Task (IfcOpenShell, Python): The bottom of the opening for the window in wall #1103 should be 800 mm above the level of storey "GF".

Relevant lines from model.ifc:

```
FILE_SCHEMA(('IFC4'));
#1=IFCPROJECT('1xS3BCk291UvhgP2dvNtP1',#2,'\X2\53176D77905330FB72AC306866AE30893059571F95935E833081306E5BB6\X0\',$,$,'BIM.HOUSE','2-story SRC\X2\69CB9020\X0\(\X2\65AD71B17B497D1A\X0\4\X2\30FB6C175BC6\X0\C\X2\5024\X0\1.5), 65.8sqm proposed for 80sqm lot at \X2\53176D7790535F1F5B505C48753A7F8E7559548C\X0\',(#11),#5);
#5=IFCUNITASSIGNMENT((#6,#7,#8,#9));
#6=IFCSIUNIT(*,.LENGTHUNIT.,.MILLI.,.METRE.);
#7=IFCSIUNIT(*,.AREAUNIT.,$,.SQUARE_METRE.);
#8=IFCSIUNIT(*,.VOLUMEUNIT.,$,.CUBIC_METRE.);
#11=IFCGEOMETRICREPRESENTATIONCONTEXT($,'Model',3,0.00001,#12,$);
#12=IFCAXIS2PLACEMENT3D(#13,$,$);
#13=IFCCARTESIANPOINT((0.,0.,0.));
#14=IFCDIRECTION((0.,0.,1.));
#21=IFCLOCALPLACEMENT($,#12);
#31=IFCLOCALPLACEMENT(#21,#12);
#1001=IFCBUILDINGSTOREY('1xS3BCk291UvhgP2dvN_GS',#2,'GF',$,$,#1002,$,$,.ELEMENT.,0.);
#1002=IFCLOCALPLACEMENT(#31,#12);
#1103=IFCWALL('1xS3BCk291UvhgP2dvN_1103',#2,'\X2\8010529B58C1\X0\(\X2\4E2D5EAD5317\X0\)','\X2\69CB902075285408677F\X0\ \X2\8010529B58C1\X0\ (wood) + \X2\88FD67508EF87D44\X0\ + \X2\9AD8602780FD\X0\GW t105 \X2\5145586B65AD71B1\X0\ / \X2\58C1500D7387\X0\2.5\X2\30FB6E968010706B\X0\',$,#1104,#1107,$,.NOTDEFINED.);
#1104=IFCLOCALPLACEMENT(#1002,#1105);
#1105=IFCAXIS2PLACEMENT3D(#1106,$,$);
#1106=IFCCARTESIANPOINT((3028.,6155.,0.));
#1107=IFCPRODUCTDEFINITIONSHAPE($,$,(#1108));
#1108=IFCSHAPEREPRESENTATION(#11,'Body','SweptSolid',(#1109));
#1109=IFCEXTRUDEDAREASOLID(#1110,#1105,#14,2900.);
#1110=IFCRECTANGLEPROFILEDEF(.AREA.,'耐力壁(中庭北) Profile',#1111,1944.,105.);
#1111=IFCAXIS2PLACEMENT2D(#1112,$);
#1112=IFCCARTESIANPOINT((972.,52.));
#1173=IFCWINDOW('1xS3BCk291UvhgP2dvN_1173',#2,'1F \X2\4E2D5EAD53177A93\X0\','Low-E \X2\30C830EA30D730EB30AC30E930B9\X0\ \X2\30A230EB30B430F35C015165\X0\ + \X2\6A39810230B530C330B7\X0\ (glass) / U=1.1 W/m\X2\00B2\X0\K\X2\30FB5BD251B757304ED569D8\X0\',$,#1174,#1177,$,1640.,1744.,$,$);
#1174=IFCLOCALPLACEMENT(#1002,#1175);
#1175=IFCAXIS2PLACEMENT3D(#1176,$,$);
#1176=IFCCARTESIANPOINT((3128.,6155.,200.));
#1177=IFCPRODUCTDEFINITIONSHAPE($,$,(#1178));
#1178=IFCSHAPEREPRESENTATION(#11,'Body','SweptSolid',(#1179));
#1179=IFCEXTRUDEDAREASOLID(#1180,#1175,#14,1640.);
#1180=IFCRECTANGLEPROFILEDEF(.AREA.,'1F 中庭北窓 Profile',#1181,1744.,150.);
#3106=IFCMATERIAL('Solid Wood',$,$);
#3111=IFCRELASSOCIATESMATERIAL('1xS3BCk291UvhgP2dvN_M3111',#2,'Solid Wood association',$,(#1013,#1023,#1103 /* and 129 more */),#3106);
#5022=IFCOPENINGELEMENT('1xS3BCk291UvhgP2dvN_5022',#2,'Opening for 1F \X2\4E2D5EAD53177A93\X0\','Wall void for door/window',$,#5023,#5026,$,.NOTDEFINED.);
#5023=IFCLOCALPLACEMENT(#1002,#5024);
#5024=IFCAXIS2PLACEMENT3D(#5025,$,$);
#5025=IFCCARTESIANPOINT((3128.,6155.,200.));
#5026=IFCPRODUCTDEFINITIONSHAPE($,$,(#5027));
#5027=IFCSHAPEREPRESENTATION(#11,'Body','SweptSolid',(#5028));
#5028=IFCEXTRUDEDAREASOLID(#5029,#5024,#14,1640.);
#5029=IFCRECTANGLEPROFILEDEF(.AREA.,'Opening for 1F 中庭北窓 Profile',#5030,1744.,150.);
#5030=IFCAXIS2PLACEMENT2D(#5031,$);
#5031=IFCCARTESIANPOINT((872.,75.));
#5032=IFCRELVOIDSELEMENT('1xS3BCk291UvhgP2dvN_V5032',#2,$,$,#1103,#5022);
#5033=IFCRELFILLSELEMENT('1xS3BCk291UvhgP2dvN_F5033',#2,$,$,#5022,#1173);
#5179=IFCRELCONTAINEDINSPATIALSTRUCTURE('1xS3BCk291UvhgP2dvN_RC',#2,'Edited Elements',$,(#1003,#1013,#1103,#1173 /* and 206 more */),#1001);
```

```python
import numpy as np
import ifcopenshell
import ifcopenshell.api.geometry
import ifcopenshell.geom
import ifcopenshell.util.element
import ifcopenshell.util.placement
import ifcopenshell.util.shape
import ifcopenshell.util.unit

model = ifcopenshell.open("model.ifc")
unit_scale = ifcopenshell.util.unit.calculate_unit_scale(model)

window = model.by_guid("1xS3BCk291UvhgP2dvN_1173")
opening = window.FillsVoids[0].RelatingOpeningElement
storey = ifcopenshell.util.element.get_container(window, ifc_class="IfcBuildingStorey")
level = ifcopenshell.util.placement.get_local_placement(storey.ObjectPlacement)[2, 3]

# The opening's origin need not be at the sill, so measure its lowest point.
shape = ifcopenshell.geom.create_shape(ifcopenshell.geom.settings(), opening)
bottom = ifcopenshell.util.shape.get_shape_bottom_elevation(shape, shape.geometry) / unit_scale
dz = level + 0.8 / unit_scale - bottom

shift = np.array([0.0, 0.0, dz])
# The window is not placed relative to its opening, so move both.
for product in (opening, window):
    matrix = ifcopenshell.util.placement.get_local_placement(product.ObjectPlacement)
    matrix[:3, 3] += shift
    ifcopenshell.api.geometry.edit_object_placement(model, product=product, matrix=matrix, is_si=False)

print(f"moved by {dz * unit_scale:+.3f} m")

model.write("model_v2.ifc")
```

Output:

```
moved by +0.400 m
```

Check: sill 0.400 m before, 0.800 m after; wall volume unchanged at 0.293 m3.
